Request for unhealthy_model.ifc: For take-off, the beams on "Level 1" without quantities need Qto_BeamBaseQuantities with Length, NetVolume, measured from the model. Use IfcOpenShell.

First a look at what the model holds.

```python
import ifcopenshell
import ifcopenshell.util.element
import ifcopenshell.util.unit

model = ifcopenshell.open("unhealthy_model.ifc")
print(model.schema)
for unit_type in ("LENGTHUNIT", "AREAUNIT", "VOLUMEUNIT"):
    print(unit_type, ifcopenshell.util.unit.calculate_unit_scale(model, unit_type))
storey = next(s for s in model.by_type("IfcBuildingStorey") if s.Name == "Level 1")
beams = [e for e in ifcopenshell.util.element.get_decomposition(storey) if e.is_a("IfcBeam")]
for e in sorted(beams, key=lambda e: e.id()):
    print(e.id(), e.is_a(), e.Name, list(ifcopenshell.util.element.get_psets(e, qtos_only=True)), sep=" | ")
```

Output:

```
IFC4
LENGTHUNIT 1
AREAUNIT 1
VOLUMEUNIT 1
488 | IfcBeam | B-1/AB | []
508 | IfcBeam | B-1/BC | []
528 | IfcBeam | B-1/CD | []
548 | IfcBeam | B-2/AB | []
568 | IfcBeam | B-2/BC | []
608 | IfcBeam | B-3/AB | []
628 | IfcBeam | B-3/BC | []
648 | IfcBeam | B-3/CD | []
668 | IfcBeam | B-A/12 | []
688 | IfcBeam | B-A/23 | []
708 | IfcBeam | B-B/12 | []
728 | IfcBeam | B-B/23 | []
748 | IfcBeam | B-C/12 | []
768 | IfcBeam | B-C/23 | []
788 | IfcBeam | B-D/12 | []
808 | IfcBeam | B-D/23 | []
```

```python
import ifcopenshell
import ifcopenshell.api.pset
import ifcopenshell.geom
import ifcopenshell.util.element
import ifcopenshell.util.shape
import ifcopenshell.util.unit

model = ifcopenshell.open("unhealthy_model.ifc")
unit_scale = ifcopenshell.util.unit.calculate_unit_scale(model)
volume_scale = ifcopenshell.util.unit.calculate_unit_scale(model, "VOLUMEUNIT")
settings = ifcopenshell.geom.settings()

storey = next(s for s in model.by_type("IfcBuildingStorey") if s.Name == "Level 1")
beams = [e for e in ifcopenshell.util.element.get_decomposition(storey) if e.is_a("IfcBeam")]

for e in sorted(beams, key=lambda e: e.id()):
    if ifcopenshell.util.element.get_psets(e, qtos_only=True, should_inherit=False):
        continue
    # Geometry comes back in metres, in the element's own axes.
    shape = ifcopenshell.geom.create_shape(settings, e)
    values = {
        "Length": ifcopenshell.util.shape.get_max_xyz(shape.geometry) / unit_scale,
        "NetVolume": ifcopenshell.util.shape.get_volume(shape.geometry) / volume_scale,
    }
    qto = ifcopenshell.api.pset.add_qto(model, product=e, name="Qto_BeamBaseQuantities")
    ifcopenshell.api.pset.edit_qto(model, qto=qto, properties=values)
    print(e.id(), {k: round(v, 3) for k, v in values.items()})

model.write("unhealthy_model_edited.ifc")
```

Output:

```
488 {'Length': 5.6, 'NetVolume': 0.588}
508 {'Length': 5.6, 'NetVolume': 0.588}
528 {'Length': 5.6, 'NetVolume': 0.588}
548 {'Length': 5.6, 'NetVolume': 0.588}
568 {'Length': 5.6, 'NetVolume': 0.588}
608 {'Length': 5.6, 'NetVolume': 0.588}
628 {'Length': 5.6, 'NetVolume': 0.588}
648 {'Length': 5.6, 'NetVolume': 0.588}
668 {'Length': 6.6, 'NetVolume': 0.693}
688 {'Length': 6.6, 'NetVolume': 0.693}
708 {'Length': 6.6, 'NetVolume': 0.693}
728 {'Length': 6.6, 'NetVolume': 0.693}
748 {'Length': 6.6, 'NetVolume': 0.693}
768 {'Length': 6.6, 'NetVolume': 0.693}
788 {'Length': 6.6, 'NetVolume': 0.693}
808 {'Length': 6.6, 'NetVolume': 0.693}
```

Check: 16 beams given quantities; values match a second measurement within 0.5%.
